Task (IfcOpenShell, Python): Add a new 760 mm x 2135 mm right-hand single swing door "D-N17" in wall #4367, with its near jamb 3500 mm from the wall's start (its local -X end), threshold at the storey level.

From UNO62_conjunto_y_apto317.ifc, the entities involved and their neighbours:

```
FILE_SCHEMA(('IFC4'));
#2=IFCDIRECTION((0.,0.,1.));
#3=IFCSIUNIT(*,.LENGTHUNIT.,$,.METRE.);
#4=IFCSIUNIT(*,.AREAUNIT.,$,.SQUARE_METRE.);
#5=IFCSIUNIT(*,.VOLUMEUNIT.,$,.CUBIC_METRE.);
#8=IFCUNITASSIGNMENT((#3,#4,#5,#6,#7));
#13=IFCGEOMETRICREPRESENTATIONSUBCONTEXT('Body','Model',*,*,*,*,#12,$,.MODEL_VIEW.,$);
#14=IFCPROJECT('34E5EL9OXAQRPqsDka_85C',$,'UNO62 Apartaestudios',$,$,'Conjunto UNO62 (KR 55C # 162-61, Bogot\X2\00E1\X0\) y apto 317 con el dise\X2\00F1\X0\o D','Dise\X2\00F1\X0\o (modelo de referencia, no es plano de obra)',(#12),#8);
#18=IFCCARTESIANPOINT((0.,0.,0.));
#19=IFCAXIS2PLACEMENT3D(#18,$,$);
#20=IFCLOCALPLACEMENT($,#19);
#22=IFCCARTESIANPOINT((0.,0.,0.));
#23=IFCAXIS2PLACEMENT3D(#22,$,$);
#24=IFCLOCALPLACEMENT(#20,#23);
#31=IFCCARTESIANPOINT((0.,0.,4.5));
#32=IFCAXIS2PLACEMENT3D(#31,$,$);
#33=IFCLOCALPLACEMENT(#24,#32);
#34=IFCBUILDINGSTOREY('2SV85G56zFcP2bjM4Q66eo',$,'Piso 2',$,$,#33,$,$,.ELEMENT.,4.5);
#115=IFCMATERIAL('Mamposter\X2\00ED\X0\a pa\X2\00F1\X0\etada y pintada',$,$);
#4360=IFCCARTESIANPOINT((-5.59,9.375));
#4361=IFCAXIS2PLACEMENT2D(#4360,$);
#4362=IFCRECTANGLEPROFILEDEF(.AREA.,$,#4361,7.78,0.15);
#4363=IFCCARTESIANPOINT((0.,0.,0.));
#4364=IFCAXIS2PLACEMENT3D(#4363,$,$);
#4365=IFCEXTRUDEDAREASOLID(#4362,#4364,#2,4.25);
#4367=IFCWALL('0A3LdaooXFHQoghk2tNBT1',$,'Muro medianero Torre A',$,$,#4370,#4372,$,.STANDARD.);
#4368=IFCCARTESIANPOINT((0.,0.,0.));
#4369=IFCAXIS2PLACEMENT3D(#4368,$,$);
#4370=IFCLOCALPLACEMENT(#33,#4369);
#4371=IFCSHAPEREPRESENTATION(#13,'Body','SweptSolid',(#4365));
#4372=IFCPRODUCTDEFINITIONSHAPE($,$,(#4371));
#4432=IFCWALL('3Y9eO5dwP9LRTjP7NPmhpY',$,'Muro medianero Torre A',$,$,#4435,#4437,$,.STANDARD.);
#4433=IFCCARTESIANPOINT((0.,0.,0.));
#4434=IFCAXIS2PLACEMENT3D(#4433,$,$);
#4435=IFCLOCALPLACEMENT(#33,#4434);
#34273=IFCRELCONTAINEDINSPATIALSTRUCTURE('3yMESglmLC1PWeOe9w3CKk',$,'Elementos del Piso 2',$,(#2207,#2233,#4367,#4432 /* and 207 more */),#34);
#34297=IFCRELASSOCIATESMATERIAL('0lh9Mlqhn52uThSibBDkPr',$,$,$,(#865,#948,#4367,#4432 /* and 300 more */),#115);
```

```python
import numpy as np
import ifcopenshell
import ifcopenshell.api.feature
import ifcopenshell.api.geometry
import ifcopenshell.api.root
import ifcopenshell.api.spatial
import ifcopenshell.geom
import ifcopenshell.util.element
import ifcopenshell.util.placement
import ifcopenshell.util.representation
import ifcopenshell.util.shape
import ifcopenshell.util.unit

model = ifcopenshell.open("UNO62_conjunto_y_apto317.ifc")
unit_scale = ifcopenshell.util.unit.calculate_unit_scale(model)
settings = ifcopenshell.geom.settings()


def volume(element):
    """Net volume in cubic metres, openings subtracted."""
    shape = ifcopenshell.geom.create_shape(settings, element)
    return ifcopenshell.util.shape.get_volume(shape.geometry)


wall = model.by_guid("0A3LdaooXFHQoghk2tNBT1")
storey = ifcopenshell.util.element.get_container(wall, ifc_class="IfcBuildingStorey")
context = ifcopenshell.util.representation.get_context(model, "Model", "Body", "MODEL_VIEW")
before = volume(wall)

width, height, from_end, sill = 0.76, 2.135, 3.5, 0.0  # metres

# The wall runs along its own X axis, and the end named is its -X end.
wall_shape = ifcopenshell.geom.create_shape(settings, wall)
x, y, z = ifcopenshell.util.shape.get_vertices(wall_shape.geometry).T
start = x.min() + from_end
face, thickness = float(y.min()), float(y.max() - y.min())
wall_matrix = ifcopenshell.util.placement.get_local_placement(wall.ObjectPlacement)
level = ifcopenshell.util.placement.get_local_placement(storey.ObjectPlacement)[2, 3]


def in_wall(x, y):
    """Placement at x, y metres in the wall's axes, at sill height."""
    matrix = wall_matrix.copy()
    matrix[:, 3] = wall_matrix @ np.array([x / unit_scale, y / unit_scale, 0.0, 1.0])
    matrix[2, 3] = level + sill / unit_scale
    return matrix


# Opening: a box that overshoots both wall faces by 50 mm.
opening = ifcopenshell.api.root.create_entity(model, ifc_class="IfcOpeningElement", predefined_type="OPENING")
box = ifcopenshell.api.geometry.add_wall_representation(
    model, context=context, length=width, height=height, thickness=thickness + 0.1
)
ifcopenshell.api.geometry.assign_representation(model, product=opening, representation=box)
ifcopenshell.api.geometry.edit_object_placement(model, product=opening, matrix=in_wall(start, face - 0.05), is_si=False)
ifcopenshell.api.feature.add_feature(model, feature=opening, element=wall)

door = ifcopenshell.api.root.create_entity(model, ifc_class="IfcDoor", name="D-N17", predefined_type="DOOR")
door.OverallWidth, door.OverallHeight = width / unit_scale, height / unit_scale
door.OperationType = "SINGLE_SWING_RIGHT"
body = ifcopenshell.api.geometry.add_door_representation(
    model,
    context=context,
    overall_width=door.OverallWidth,
    overall_height=door.OverallHeight,
    operation_type="SINGLE_SWING_RIGHT",
    lining_properties={"LiningDepth": thickness / unit_scale, "ThresholdDepth": thickness / unit_scale},
)
ifcopenshell.api.geometry.assign_representation(model, product=door, representation=body)
ifcopenshell.api.spatial.assign_container(model, products=[door], relating_structure=storey)
ifcopenshell.api.feature.add_filling(model, opening=opening, element=door)

# The lining spans the wall, so the door starts at the wall face.
ifcopenshell.api.geometry.edit_object_placement(model, product=door, matrix=in_wall(start, face), is_si=False)

after = volume(wall)

print(f"wall volume {before:.3f} -> {after:.3f} m3")

model.write("UNO62_conjunto_y_apto317_edited.ifc")
```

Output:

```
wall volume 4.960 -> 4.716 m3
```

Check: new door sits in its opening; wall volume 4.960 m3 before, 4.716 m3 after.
